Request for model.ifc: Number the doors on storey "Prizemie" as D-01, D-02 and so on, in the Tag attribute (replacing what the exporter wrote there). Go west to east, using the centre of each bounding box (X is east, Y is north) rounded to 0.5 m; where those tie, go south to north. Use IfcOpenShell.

First a look at what the model holds.

```python
import ifcopenshell
import ifcopenshell.util.element
import ifcopenshell.util.placement

model = ifcopenshell.open("model.ifc")
print(model.schema)
storey = next(s for s in model.by_type("IfcBuildingStorey") if s.Name == "Prizemie")
doors = [e for e in ifcopenshell.util.element.get_decomposition(storey) if e.is_a("IfcDoor")]
for e in sorted(doors, key=lambda e: e.id()):
    origin = ifcopenshell.util.placement.get_local_placement(e.ObjectPlacement)[:3, 3]
    print(e.id(), e.Tag, e.Name, origin.round(2) + 0.0, sep=" | ")
```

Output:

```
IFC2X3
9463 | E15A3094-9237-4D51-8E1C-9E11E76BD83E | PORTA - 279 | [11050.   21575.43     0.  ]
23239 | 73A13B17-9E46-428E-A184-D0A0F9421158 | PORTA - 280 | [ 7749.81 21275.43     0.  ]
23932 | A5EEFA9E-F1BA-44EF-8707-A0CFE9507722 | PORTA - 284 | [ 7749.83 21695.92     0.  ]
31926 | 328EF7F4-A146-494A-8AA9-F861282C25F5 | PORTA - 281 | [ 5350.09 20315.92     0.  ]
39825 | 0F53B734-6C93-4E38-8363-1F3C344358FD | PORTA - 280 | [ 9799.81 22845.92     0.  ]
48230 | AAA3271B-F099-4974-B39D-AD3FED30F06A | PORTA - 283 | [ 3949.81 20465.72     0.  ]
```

```python
import ifcopenshell
import ifcopenshell.geom
import ifcopenshell.util.element
import ifcopenshell.util.shape

model = ifcopenshell.open("model.ifc")
settings = ifcopenshell.geom.settings()
settings.set("use-world-coords", True)


def centre(element):
    shape = ifcopenshell.geom.create_shape(settings, element)
    return ifcopenshell.util.shape.get_bbox_centroid(shape.geometry)


storey = next(s for s in model.by_type("IfcBuildingStorey") if s.Name == "Prizemie")
doors = [e for e in ifcopenshell.util.element.get_decomposition(storey) if e.is_a("IfcDoor")]

# Insertion points can sit at a corner or the storey origin, so sort by the geometry (in metres).
centres = {e: centre(e) for e in doors}
doors.sort(key=lambda e: (round(centres[e][0] / 0.5), centres[e][1]))

for i, e in enumerate(doors, start=1):
    number = f"D-{i:02d}"
    e.Tag = number
    print(e.id(), number)

model.write("model_rev.ifc")
```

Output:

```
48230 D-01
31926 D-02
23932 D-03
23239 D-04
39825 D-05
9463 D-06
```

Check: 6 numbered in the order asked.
